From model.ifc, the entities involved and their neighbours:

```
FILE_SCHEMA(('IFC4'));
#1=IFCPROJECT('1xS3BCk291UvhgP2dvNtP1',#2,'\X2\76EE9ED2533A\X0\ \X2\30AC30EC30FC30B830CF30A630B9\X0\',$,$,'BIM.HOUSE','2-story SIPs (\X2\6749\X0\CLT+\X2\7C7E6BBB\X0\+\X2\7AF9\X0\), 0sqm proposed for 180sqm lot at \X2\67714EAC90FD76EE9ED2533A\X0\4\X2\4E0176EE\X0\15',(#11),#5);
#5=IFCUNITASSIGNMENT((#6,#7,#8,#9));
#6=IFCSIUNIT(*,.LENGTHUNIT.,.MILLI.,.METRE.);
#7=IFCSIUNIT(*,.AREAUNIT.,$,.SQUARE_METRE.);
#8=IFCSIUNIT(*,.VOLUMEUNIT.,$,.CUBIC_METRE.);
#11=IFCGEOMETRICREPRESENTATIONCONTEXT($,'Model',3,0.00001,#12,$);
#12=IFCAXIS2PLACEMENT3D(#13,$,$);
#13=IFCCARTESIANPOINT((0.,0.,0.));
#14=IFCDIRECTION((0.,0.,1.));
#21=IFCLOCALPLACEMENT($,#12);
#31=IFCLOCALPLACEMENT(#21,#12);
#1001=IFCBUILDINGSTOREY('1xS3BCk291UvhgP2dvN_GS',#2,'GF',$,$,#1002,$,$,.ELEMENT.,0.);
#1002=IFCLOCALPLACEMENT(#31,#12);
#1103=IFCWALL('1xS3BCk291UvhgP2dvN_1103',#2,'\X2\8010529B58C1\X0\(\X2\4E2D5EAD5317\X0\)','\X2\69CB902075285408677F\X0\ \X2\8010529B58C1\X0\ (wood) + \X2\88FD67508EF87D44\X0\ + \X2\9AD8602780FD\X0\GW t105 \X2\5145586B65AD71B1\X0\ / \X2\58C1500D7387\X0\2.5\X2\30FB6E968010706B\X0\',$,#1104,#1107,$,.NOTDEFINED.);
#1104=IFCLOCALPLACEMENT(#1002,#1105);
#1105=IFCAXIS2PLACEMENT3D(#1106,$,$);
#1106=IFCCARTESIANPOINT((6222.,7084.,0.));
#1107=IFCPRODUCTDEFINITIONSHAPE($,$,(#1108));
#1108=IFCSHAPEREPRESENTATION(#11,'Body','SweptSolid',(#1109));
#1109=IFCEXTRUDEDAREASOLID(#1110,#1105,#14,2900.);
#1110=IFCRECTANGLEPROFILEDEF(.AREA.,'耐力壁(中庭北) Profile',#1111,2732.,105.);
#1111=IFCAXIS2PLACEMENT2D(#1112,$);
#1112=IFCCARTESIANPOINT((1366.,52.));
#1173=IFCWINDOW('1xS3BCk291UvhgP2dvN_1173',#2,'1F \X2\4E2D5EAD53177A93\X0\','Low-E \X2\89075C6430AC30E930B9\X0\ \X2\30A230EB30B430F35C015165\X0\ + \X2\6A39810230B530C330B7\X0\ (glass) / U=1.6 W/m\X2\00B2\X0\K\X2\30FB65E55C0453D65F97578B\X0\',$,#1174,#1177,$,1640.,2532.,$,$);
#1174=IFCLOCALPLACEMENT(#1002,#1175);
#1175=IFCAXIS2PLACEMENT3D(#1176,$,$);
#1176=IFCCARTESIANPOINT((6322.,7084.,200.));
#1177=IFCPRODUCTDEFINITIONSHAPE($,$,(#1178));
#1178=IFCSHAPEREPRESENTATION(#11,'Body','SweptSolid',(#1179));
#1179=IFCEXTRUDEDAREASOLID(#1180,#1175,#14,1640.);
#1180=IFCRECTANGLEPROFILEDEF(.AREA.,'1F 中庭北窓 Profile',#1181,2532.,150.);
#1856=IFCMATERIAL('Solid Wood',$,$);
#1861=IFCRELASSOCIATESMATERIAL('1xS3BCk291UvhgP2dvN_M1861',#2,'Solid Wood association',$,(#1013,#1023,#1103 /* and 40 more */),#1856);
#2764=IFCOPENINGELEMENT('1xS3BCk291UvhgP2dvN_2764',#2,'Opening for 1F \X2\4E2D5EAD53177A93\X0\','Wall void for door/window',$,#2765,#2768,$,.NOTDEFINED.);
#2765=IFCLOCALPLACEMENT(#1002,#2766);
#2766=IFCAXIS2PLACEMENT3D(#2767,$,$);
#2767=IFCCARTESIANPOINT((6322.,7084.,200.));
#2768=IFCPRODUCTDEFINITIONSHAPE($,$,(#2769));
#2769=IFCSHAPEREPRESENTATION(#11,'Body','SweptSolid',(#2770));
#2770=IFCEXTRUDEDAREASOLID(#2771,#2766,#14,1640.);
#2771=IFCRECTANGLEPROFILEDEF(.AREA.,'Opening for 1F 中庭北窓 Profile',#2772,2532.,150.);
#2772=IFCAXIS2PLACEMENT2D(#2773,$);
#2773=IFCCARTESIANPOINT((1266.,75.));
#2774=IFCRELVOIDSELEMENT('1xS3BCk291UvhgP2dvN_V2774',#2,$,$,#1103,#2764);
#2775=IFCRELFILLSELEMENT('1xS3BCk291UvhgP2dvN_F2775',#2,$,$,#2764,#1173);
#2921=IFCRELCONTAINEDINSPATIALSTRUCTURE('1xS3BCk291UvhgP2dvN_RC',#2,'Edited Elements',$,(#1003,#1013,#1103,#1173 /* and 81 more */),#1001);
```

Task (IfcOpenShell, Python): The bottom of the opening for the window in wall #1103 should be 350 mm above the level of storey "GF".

```python
import numpy as np
import ifcopenshell
import ifcopenshell.api.geometry
import ifcopenshell.geom
import ifcopenshell.util.element
import ifcopenshell.util.placement
import ifcopenshell.util.shape
import ifcopenshell.util.unit

model = ifcopenshell.open("model.ifc")
unit_scale = ifcopenshell.util.unit.calculate_unit_scale(model)

window = model.by_id(1173)
opening = window.FillsVoids[0].RelatingOpeningElement
storey = ifcopenshell.util.element.get_container(window, ifc_class="IfcBuildingStorey")
level = ifcopenshell.util.placement.get_local_placement(storey.ObjectPlacement)[2, 3]

# The opening's origin need not be at the sill, so measure its lowest point.
shape = ifcopenshell.geom.create_shape(ifcopenshell.geom.settings(), opening)
bottom = ifcopenshell.util.shape.get_shape_bottom_elevation(shape, shape.geometry) / unit_scale
dz = level + 0.35 / unit_scale - bottom

shift = np.array([0.0, 0.0, dz])
# The window is not placed relative to its opening, so move both.
for product in (opening, window):
    matrix = ifcopenshell.util.placement.get_local_placement(product.ObjectPlacement)
    matrix[:3, 3] += shift
    ifcopenshell.api.geometry.edit_object_placement(model, product=product, matrix=matrix, is_si=False)

print(f"moved by {dz * unit_scale:+.3f} m")

model.write("model-out.ifc")
```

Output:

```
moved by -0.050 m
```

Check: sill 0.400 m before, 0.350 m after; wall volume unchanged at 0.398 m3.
